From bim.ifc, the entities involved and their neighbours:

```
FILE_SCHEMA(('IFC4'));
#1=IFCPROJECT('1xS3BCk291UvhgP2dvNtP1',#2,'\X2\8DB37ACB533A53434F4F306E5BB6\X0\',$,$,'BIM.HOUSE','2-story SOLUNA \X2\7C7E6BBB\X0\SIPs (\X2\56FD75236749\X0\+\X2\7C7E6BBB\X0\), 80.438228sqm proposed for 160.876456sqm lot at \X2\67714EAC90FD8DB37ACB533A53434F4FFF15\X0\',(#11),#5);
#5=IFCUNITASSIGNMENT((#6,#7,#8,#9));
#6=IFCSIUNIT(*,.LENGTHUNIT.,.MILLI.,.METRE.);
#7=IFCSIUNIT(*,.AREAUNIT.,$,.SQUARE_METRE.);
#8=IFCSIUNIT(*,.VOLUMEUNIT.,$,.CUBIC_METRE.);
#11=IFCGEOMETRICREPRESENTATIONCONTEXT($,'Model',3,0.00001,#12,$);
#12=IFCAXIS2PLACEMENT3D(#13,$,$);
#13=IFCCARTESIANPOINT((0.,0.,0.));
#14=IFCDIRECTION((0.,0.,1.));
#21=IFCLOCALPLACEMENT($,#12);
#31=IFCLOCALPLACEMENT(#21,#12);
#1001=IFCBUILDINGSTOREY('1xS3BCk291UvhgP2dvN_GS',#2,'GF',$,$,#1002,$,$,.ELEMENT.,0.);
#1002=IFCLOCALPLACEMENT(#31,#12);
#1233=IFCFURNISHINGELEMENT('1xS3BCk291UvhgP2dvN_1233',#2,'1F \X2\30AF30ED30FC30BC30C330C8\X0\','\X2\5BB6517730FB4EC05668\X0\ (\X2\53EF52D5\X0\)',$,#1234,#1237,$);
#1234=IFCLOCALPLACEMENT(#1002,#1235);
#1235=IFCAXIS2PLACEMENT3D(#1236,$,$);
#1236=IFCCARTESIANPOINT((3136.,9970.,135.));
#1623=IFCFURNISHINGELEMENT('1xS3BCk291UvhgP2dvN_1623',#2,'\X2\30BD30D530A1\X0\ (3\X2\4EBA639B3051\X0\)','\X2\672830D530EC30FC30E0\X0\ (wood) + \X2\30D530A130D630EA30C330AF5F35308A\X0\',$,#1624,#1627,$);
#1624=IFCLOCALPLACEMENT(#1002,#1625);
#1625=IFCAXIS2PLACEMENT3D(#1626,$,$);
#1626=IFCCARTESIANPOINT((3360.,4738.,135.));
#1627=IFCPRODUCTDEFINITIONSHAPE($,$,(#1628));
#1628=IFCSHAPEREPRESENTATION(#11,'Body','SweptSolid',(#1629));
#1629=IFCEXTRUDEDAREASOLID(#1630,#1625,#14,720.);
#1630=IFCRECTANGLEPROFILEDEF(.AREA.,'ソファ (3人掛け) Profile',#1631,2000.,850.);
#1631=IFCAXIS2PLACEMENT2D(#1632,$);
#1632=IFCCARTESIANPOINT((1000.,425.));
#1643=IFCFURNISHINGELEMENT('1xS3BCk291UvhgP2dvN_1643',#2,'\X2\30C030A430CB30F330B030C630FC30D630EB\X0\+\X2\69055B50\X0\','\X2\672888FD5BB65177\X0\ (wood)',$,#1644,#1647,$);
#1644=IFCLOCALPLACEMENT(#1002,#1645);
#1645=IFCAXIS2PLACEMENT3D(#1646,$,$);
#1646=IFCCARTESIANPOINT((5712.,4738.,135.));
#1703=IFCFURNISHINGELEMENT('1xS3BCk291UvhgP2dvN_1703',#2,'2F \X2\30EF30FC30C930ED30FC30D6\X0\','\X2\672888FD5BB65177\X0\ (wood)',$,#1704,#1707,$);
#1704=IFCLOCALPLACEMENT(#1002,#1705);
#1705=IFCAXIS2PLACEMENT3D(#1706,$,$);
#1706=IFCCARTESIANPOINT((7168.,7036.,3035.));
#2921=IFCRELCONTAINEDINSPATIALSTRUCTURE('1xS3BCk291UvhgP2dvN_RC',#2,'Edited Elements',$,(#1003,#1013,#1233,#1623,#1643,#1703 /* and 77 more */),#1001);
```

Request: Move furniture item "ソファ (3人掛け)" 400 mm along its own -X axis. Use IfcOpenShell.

```python
import ifcopenshell
import ifcopenshell.api.geometry
import ifcopenshell.util.placement
import ifcopenshell.util.unit

model = ifcopenshell.open("bim.ifc")
unit_scale = ifcopenshell.util.unit.calculate_unit_scale(model)

item = model.by_guid("1xS3BCk291UvhgP2dvN_1623")
matrix = ifcopenshell.util.placement.get_local_placement(item.ObjectPlacement)
matrix[:3, 3] -= matrix[:3, 0] * 0.4 / unit_scale
ifcopenshell.api.geometry.edit_object_placement(model, product=item, matrix=matrix, is_si=False)

print(ifcopenshell.util.placement.get_local_placement(item.ObjectPlacement).round(3) + 0.0)

model.write("bim_rev.ifc")
```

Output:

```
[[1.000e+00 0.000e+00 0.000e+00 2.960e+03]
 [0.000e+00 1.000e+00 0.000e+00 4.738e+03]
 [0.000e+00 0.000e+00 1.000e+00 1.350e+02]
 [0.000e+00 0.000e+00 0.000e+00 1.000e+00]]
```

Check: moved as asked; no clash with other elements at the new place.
